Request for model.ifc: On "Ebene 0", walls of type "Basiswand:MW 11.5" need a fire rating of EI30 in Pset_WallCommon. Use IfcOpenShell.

First a look at what the model holds.

```python
import ifcopenshell
import ifcopenshell.util.element

model = ifcopenshell.open("model.ifc")
print(model.schema)
storey = next(s for s in model.by_type("IfcBuildingStorey") if s.Name == "Ebene 0")
walls = [e for e in ifcopenshell.util.element.get_decomposition(storey) if e.is_a("IfcWall")]
seen = {}
for e in walls:
    element_type = ifcopenshell.util.element.get_type(e)
    key = (element_type.Name if element_type != e and element_type else None, ifcopenshell.util.element.get_pset(e, "Pset_WallCommon", "FireRating"))
    seen[key] = seen.get(key, 0) + 1
for (name, value), count in sorted(seen.items(), key=str):
    print(count, "x", name, "|", value)
```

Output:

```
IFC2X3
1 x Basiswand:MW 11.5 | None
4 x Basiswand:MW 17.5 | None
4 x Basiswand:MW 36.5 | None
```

```python
import ifcopenshell
import ifcopenshell.api.pset
import ifcopenshell.util.element

model = ifcopenshell.open("model.ifc")

storey = next(s for s in model.by_type("IfcBuildingStorey") if s.Name == "Ebene 0")
walls = [e for e in ifcopenshell.util.element.get_decomposition(storey) if e.is_a("IfcWall")]

count = 0
for e in walls:
    element_type = ifcopenshell.util.element.get_type(e)
    if element_type in (None, e) or element_type.Name != "Basiswand:MW 11.5":
        continue
    # add_pset returns the element's existing set when there is one.
    pset = ifcopenshell.api.pset.add_pset(model, product=e, name="Pset_WallCommon")
    ifcopenshell.api.pset.edit_pset(model, pset=pset, properties={"FireRating": "EI30"})
    count += 1

print(count, "walls updated")

model.write("model_v2.ifc")
```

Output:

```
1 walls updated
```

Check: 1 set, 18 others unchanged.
